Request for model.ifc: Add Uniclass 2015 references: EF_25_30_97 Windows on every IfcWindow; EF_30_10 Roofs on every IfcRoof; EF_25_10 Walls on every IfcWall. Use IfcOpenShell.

First a look at what the model holds.

```python
import ifcopenshell

model = ifcopenshell.open("model.ifc")
print(model.schema)
print("classifications:", [c.Name for c in model.by_type("IfcClassification")])
for ifc_class in ("IfcDoor", "IfcRoof", "IfcStair", "IfcWall", "IfcWindow"):
    print(ifc_class, len(model.by_type(ifc_class)))
```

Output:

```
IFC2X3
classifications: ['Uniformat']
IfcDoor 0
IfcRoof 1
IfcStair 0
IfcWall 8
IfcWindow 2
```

```python
import ifcopenshell
import ifcopenshell.api.classification

model = ifcopenshell.open("model.ifc")

# IFC2X3 requires Source and Edition and has no link from the project to the system.
system = model.create_entity("IfcClassification", Source="NBS", Edition="2015", Name="Uniclass 2015")

codes = {
    "IfcWindow": ("EF_25_30_97", "Windows"),
    "IfcRoof": ("EF_30_10", "Roofs"),
    "IfcWall": ("EF_25_10", "Walls"),
}
for ifc_class, (code, name) in codes.items():
    products = model.by_type(ifc_class)
    ifcopenshell.api.classification.add_reference(
        model, products=products, classification=system, identification=code, name=name
    )
    print(code, len(products))

model.write("model_rev.ifc")
```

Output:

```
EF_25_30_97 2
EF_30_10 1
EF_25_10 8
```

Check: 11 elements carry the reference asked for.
